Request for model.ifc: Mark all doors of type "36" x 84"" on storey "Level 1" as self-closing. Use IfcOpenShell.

First a look at what the model holds.

```python
import ifcopenshell
import ifcopenshell.util.element

model = ifcopenshell.open("model.ifc")
print(model.schema)
storey = next(s for s in model.by_type("IfcBuildingStorey") if s.Name == "Level 1")
doors = [e for e in ifcopenshell.util.element.get_decomposition(storey) if e.is_a("IfcDoor")]
seen = {}
for e in doors:
    element_type = ifcopenshell.util.element.get_type(e)
    key = (element_type.Name if element_type != e and element_type else None, ifcopenshell.util.element.get_pset(e, "Pset_DoorCommon", "SelfClosing"))
    seen[key] = seen.get(key, 0) + 1
for (name, value), count in sorted(seen.items(), key=str):
    print(count, "x", name, "|", value)
```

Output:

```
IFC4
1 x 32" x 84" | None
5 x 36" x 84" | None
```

```python
import ifcopenshell
import ifcopenshell.api.pset
import ifcopenshell.util.element

model = ifcopenshell.open("model.ifc")

storey = next(s for s in model.by_type("IfcBuildingStorey") if s.Name == "Level 1")
doors = [e for e in ifcopenshell.util.element.get_decomposition(storey) if e.is_a("IfcDoor")]

count = 0
for e in doors:
    element_type = ifcopenshell.util.element.get_type(e)
    if element_type in (None, e) or element_type.Name != '36" x 84"':
        continue
    # add_pset returns the element's existing set when there is one.
    pset = ifcopenshell.api.pset.add_pset(model, product=e, name="Pset_DoorCommon")
    ifcopenshell.api.pset.edit_pset(model, pset=pset, properties={"SelfClosing": True})
    count += 1

print(count, "doors updated")

model.write("model_rev.ifc")
```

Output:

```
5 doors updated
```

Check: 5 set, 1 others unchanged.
